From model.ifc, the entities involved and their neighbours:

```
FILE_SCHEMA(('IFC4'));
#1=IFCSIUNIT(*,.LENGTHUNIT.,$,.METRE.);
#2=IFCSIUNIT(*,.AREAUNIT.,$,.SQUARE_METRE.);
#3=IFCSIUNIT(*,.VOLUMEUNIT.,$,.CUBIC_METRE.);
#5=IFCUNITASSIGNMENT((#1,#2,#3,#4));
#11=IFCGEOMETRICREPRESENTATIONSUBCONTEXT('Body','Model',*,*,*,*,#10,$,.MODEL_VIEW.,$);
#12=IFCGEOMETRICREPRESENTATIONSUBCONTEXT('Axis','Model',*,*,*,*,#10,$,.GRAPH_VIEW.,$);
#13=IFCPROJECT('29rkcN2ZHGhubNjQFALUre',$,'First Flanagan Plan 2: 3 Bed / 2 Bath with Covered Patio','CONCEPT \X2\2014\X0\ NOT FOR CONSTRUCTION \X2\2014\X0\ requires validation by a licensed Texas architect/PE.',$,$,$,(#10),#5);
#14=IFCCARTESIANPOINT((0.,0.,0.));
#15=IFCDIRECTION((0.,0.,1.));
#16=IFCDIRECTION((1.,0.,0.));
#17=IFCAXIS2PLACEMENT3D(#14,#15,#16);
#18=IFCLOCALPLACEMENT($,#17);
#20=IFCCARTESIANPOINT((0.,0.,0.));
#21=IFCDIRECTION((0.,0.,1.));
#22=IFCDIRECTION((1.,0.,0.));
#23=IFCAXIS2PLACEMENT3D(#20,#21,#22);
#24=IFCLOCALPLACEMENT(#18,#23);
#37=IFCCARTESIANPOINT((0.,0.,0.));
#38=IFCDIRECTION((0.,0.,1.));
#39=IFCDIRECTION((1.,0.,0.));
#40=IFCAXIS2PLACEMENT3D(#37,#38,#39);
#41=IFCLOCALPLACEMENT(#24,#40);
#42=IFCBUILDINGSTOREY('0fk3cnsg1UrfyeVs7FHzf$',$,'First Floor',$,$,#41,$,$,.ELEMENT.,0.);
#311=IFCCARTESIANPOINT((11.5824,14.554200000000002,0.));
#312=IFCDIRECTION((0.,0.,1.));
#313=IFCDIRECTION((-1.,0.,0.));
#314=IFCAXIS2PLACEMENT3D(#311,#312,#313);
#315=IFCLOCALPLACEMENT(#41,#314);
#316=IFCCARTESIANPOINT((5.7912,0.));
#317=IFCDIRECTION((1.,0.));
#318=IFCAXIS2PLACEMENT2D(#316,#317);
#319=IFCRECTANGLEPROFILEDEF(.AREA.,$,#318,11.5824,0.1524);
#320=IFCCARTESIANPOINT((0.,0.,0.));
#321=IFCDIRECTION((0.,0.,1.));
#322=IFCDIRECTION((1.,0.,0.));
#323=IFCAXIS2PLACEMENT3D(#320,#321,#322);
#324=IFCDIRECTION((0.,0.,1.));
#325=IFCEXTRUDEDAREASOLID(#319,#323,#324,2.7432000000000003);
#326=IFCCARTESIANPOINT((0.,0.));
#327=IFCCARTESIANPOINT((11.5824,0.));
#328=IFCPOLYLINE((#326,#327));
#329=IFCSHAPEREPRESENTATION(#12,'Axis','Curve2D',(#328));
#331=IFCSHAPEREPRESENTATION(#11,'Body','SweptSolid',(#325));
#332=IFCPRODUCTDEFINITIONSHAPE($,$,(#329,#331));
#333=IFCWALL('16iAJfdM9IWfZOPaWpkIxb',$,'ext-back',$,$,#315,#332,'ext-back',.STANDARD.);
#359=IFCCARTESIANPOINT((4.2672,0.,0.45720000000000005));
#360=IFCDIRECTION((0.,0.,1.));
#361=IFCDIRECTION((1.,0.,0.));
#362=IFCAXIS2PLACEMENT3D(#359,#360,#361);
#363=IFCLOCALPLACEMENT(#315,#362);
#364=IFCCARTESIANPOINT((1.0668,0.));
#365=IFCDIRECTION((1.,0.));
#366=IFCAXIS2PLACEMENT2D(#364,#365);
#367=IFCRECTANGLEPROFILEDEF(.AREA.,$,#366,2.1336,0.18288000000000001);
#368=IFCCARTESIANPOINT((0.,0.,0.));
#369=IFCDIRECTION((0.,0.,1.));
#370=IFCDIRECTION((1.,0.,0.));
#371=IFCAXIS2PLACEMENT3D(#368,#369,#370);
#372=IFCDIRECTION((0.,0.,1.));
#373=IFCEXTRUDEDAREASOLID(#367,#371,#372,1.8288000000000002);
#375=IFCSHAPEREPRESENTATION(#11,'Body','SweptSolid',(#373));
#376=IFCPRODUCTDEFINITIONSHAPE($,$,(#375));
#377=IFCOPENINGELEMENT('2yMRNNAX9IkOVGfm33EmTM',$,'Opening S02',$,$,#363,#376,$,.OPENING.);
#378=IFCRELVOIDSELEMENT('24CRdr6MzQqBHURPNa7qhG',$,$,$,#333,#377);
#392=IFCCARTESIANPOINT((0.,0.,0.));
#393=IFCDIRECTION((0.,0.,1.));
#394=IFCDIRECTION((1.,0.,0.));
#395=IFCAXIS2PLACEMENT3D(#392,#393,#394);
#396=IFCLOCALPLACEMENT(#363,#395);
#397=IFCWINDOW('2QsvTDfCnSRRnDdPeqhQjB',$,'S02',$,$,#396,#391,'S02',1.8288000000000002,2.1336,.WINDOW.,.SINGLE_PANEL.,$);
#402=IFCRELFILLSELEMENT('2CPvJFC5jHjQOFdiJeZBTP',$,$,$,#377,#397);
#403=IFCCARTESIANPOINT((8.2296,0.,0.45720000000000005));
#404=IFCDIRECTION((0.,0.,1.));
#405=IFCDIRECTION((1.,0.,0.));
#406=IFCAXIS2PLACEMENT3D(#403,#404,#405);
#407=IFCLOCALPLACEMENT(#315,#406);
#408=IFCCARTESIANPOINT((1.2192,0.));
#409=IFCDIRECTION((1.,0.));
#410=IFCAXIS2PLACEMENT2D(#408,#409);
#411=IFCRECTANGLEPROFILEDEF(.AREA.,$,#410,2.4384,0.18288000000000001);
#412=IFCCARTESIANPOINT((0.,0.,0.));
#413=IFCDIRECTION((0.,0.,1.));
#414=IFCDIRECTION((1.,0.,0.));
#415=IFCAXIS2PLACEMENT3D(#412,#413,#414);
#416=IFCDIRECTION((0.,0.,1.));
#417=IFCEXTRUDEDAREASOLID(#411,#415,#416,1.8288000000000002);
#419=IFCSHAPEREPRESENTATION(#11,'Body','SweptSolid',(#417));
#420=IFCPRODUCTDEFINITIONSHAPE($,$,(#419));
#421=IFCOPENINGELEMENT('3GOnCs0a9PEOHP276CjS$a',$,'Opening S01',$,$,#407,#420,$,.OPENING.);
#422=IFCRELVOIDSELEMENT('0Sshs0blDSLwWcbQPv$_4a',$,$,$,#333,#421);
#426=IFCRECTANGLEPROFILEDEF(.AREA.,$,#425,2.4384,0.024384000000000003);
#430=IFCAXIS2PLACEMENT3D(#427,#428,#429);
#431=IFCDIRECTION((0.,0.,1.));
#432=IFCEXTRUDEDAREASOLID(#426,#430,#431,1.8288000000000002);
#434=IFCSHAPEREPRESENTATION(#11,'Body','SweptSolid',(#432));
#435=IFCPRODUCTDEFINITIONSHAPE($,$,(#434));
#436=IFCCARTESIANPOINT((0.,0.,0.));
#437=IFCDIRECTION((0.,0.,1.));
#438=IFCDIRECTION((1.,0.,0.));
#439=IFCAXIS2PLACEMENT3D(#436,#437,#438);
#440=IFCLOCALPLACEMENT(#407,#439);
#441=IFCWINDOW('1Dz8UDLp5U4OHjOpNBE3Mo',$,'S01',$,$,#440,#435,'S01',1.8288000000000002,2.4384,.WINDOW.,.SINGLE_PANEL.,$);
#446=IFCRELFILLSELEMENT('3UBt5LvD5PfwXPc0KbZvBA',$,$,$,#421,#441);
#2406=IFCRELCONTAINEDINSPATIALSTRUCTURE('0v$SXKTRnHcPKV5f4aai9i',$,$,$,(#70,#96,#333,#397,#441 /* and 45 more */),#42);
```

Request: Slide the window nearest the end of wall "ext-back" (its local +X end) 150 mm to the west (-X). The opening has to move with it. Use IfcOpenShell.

```python
import ifcopenshell
import ifcopenshell.api.geometry
import ifcopenshell.util.placement
import ifcopenshell.util.unit

model = ifcopenshell.open("model.ifc")
unit_scale = ifcopenshell.util.unit.calculate_unit_scale(model)

window = model.by_guid("1Dz8UDLp5U4OHjOpNBE3Mo")
opening = window.FillsVoids[0].RelatingOpeningElement
wall = opening.VoidsElements[0].RelatingBuildingElement

wall_matrix = ifcopenshell.util.placement.get_local_placement(wall.ObjectPlacement)
shift = wall_matrix[:3, 0] * 0.15 / unit_scale
before = ifcopenshell.util.placement.get_local_placement(window.ObjectPlacement)[:3, 3].copy()

# The window is placed relative to its opening, so it follows when the opening moves.
matrix = ifcopenshell.util.placement.get_local_placement(opening.ObjectPlacement)
matrix[:3, 3] += shift
ifcopenshell.api.geometry.edit_object_placement(
    model, product=opening, matrix=matrix, is_si=False, should_transform_children=True
)

after = ifcopenshell.util.placement.get_local_placement(window.ObjectPlacement)[:3, 3]
print("window moved by", (after - before).round(3) + 0.0)

model.write("model_edited.ifc")
```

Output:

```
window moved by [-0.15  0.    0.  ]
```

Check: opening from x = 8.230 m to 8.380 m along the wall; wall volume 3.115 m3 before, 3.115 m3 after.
